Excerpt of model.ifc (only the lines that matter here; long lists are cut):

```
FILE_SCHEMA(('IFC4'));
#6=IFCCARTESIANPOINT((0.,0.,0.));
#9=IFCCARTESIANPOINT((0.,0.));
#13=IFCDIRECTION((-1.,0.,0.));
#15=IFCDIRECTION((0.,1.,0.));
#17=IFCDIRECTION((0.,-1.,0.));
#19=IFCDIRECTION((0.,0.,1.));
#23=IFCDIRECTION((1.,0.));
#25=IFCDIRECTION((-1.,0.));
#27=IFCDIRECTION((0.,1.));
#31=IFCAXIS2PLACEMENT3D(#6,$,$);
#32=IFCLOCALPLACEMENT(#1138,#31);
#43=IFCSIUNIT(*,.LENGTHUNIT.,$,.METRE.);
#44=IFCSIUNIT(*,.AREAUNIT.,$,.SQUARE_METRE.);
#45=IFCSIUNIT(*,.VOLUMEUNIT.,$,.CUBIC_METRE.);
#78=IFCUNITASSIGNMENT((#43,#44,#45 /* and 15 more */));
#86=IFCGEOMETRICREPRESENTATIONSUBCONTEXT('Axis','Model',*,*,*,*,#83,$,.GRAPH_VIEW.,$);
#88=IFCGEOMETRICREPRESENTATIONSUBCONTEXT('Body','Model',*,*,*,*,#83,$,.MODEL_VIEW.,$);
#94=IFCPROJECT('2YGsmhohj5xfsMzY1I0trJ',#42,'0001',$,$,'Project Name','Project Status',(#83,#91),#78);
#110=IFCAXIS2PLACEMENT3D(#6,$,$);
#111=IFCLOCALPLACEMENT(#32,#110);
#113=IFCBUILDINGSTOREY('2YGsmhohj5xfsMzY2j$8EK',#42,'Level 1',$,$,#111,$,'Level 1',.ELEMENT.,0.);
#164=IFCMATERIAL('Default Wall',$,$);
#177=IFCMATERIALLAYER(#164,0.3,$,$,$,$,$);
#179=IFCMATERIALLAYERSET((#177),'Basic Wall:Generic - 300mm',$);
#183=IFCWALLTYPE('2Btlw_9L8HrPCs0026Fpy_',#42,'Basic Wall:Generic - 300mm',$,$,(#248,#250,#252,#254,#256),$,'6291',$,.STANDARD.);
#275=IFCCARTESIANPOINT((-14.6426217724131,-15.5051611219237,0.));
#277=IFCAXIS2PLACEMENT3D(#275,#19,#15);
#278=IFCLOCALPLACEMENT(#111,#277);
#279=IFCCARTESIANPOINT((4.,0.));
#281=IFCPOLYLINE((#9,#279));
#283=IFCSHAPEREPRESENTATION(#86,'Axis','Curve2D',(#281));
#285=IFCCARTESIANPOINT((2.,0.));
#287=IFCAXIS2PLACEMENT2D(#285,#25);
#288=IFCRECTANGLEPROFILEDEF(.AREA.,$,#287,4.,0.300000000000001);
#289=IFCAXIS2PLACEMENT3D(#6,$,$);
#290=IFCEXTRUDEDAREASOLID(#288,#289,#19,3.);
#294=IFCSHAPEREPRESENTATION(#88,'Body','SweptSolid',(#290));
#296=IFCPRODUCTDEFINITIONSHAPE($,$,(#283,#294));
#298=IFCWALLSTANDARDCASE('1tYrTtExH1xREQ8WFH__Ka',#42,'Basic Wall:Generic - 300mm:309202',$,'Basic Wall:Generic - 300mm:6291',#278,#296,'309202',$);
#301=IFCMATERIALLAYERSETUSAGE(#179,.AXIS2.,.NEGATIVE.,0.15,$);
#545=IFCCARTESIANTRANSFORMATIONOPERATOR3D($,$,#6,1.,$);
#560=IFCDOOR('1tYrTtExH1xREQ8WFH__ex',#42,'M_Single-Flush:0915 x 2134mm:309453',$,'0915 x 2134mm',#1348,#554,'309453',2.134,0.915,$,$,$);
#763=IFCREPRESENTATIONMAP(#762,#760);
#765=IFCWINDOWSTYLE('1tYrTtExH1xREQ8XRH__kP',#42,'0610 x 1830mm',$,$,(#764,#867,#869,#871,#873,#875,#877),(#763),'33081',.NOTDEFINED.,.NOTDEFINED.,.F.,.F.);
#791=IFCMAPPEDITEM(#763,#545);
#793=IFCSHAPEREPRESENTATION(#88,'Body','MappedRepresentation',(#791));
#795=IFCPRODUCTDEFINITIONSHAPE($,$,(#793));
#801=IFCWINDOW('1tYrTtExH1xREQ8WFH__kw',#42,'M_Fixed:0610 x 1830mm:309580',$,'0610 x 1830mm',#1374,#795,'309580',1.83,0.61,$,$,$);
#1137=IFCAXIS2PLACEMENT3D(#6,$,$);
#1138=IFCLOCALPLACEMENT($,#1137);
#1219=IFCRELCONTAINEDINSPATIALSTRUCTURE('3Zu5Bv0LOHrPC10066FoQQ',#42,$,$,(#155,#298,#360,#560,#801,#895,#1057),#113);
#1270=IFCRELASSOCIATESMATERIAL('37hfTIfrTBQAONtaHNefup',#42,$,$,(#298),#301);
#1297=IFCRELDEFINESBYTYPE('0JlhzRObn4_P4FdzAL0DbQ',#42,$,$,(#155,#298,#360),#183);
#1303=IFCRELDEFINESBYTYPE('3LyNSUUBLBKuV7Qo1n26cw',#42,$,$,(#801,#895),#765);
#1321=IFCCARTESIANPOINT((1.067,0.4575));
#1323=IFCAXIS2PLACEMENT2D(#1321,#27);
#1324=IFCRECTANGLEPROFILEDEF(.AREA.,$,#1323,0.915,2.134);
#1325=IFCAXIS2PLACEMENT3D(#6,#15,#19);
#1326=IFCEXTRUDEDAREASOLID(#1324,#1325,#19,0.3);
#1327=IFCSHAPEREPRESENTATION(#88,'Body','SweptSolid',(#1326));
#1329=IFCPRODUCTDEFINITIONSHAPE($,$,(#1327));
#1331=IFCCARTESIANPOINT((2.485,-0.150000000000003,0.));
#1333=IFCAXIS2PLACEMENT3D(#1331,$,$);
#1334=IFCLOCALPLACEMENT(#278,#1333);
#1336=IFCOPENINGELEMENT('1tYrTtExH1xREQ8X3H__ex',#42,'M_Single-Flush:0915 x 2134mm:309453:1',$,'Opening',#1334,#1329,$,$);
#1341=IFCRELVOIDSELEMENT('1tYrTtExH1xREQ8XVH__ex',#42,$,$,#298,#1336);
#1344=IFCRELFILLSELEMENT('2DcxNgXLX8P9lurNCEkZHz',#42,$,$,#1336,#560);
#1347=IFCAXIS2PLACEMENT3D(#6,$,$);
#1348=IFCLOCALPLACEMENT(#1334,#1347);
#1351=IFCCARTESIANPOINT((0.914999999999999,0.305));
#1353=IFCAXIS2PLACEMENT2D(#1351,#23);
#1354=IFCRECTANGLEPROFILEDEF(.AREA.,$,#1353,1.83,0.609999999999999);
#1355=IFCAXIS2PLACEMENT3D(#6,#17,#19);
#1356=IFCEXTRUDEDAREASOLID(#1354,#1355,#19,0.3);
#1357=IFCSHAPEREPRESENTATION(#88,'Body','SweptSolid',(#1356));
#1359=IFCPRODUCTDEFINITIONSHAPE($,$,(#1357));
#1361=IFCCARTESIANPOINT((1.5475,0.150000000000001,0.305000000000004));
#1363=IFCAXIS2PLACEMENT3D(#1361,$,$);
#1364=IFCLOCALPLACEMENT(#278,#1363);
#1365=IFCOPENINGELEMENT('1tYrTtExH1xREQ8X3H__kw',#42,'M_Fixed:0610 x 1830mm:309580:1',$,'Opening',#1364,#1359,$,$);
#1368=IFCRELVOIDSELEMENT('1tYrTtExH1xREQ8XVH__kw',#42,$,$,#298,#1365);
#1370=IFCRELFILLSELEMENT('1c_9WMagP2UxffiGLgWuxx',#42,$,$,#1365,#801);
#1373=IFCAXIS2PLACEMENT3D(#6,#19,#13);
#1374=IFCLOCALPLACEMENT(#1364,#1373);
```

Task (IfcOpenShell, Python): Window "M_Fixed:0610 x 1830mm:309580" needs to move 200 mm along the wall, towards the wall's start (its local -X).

```python
import ifcopenshell
import ifcopenshell.api.geometry
import ifcopenshell.util.placement
import ifcopenshell.util.unit

model = ifcopenshell.open("model.ifc")
unit_scale = ifcopenshell.util.unit.calculate_unit_scale(model)

window = model.by_id(801)
opening = window.FillsVoids[0].RelatingOpeningElement
wall = opening.VoidsElements[0].RelatingBuildingElement

wall_matrix = ifcopenshell.util.placement.get_local_placement(wall.ObjectPlacement)
shift = wall_matrix[:3, 0] * -0.2 / unit_scale
before = ifcopenshell.util.placement.get_local_placement(window.ObjectPlacement)[:3, 3].copy()

# The window is placed relative to its opening, so it follows when the opening moves.
matrix = ifcopenshell.util.placement.get_local_placement(opening.ObjectPlacement)
matrix[:3, 3] += shift
ifcopenshell.api.geometry.edit_object_placement(
    model, product=opening, matrix=matrix, is_si=False, should_transform_children=True
)

after = ifcopenshell.util.placement.get_local_placement(window.ObjectPlacement)[:3, 3]
print("window moved by", (after - before).round(3) + 0.0)

model.write("model_v2.ifc")
```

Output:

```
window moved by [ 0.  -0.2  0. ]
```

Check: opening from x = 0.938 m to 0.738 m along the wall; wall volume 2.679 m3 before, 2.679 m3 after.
